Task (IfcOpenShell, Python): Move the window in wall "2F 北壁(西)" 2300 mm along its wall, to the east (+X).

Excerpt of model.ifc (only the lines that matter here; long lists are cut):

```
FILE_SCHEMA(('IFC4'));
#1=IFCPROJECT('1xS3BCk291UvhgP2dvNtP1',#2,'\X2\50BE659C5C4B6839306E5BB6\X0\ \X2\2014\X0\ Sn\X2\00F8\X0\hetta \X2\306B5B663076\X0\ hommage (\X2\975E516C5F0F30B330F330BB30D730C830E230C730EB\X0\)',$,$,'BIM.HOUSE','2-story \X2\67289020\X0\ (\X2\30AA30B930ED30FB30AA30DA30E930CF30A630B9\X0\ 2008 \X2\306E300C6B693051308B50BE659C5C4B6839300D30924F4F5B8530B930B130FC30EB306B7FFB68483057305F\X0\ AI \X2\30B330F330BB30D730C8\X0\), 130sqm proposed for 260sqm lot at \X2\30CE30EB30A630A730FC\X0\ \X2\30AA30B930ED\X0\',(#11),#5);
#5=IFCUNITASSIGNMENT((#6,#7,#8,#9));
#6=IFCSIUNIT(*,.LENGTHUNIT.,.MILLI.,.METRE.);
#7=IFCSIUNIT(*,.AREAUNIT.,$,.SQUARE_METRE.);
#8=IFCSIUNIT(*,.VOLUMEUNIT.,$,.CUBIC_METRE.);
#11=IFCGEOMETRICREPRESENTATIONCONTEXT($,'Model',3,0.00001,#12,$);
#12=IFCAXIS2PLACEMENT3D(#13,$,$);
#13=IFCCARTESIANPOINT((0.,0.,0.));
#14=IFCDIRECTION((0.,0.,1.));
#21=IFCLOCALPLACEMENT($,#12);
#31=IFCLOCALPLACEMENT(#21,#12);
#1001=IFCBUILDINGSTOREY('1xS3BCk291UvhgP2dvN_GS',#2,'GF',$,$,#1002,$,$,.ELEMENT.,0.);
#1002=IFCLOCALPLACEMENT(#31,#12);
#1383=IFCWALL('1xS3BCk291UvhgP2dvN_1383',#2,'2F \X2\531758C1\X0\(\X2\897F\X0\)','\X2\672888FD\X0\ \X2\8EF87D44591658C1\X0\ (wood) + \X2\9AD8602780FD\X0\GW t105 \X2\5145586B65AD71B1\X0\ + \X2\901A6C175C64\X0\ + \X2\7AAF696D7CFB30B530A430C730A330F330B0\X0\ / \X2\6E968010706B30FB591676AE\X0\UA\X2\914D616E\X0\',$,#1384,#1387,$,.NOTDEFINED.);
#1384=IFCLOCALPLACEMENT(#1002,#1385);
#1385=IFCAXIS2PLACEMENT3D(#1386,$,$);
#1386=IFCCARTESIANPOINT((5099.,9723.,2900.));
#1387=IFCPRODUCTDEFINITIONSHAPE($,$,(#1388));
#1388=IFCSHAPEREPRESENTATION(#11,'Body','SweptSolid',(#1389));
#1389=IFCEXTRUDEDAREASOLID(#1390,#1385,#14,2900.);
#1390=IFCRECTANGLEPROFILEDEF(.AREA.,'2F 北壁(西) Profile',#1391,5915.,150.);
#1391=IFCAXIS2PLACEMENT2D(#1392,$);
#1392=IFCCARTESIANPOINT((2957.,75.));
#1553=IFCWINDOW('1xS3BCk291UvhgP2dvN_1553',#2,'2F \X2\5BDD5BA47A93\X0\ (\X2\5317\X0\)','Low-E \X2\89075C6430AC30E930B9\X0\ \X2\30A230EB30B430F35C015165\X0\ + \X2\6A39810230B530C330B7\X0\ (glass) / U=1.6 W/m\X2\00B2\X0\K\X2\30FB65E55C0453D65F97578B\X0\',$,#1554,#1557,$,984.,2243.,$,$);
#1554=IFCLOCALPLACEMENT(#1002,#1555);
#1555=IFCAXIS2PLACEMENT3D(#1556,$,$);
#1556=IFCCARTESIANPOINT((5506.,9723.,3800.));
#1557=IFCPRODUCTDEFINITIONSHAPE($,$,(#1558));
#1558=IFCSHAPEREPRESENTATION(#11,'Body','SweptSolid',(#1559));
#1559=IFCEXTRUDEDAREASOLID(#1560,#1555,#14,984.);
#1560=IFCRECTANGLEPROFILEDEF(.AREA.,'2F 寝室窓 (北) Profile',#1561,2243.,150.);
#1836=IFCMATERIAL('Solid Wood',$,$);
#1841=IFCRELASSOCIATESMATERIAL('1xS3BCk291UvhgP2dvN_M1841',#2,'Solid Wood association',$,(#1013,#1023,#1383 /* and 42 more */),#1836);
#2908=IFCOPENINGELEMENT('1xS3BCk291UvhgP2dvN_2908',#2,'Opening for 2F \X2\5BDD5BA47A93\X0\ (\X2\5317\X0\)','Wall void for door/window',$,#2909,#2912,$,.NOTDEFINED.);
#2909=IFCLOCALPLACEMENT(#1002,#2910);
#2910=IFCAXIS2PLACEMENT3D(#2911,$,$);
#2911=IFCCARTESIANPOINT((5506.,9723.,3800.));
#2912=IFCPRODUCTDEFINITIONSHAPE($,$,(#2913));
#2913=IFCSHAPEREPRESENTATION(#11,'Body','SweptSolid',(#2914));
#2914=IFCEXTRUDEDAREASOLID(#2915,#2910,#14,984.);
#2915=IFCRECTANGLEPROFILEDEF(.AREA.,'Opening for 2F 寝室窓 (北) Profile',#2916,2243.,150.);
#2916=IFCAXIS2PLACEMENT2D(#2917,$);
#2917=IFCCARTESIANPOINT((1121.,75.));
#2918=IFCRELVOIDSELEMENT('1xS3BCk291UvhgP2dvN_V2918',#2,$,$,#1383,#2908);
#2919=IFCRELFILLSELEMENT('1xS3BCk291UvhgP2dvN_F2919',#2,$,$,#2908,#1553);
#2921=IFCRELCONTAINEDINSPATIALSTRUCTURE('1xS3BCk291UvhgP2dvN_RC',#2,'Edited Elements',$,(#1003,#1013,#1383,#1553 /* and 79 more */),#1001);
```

```python
import ifcopenshell
import ifcopenshell.api.geometry
import ifcopenshell.util.placement
import ifcopenshell.util.unit

model = ifcopenshell.open("model.ifc")
unit_scale = ifcopenshell.util.unit.calculate_unit_scale(model)

window = model.by_guid("1xS3BCk291UvhgP2dvN_1553")
opening = window.FillsVoids[0].RelatingOpeningElement
wall = opening.VoidsElements[0].RelatingBuildingElement

wall_matrix = ifcopenshell.util.placement.get_local_placement(wall.ObjectPlacement)
shift = wall_matrix[:3, 0] * 2.3 / unit_scale
before = ifcopenshell.util.placement.get_local_placement(window.ObjectPlacement)[:3, 3].copy()

# The window is not placed relative to its opening, so move both.
for product in (opening, window):
    matrix = ifcopenshell.util.placement.get_local_placement(product.ObjectPlacement)
    matrix[:3, 3] += shift
    ifcopenshell.api.geometry.edit_object_placement(model, product=product, matrix=matrix, is_si=False)

after = ifcopenshell.util.placement.get_local_placement(window.ObjectPlacement)[:3, 3]
print("window moved by", (after - before).round(3) + 0.0)

model.write("model_edited.ifc")
```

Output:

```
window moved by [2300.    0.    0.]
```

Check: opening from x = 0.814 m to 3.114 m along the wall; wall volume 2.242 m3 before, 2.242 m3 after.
